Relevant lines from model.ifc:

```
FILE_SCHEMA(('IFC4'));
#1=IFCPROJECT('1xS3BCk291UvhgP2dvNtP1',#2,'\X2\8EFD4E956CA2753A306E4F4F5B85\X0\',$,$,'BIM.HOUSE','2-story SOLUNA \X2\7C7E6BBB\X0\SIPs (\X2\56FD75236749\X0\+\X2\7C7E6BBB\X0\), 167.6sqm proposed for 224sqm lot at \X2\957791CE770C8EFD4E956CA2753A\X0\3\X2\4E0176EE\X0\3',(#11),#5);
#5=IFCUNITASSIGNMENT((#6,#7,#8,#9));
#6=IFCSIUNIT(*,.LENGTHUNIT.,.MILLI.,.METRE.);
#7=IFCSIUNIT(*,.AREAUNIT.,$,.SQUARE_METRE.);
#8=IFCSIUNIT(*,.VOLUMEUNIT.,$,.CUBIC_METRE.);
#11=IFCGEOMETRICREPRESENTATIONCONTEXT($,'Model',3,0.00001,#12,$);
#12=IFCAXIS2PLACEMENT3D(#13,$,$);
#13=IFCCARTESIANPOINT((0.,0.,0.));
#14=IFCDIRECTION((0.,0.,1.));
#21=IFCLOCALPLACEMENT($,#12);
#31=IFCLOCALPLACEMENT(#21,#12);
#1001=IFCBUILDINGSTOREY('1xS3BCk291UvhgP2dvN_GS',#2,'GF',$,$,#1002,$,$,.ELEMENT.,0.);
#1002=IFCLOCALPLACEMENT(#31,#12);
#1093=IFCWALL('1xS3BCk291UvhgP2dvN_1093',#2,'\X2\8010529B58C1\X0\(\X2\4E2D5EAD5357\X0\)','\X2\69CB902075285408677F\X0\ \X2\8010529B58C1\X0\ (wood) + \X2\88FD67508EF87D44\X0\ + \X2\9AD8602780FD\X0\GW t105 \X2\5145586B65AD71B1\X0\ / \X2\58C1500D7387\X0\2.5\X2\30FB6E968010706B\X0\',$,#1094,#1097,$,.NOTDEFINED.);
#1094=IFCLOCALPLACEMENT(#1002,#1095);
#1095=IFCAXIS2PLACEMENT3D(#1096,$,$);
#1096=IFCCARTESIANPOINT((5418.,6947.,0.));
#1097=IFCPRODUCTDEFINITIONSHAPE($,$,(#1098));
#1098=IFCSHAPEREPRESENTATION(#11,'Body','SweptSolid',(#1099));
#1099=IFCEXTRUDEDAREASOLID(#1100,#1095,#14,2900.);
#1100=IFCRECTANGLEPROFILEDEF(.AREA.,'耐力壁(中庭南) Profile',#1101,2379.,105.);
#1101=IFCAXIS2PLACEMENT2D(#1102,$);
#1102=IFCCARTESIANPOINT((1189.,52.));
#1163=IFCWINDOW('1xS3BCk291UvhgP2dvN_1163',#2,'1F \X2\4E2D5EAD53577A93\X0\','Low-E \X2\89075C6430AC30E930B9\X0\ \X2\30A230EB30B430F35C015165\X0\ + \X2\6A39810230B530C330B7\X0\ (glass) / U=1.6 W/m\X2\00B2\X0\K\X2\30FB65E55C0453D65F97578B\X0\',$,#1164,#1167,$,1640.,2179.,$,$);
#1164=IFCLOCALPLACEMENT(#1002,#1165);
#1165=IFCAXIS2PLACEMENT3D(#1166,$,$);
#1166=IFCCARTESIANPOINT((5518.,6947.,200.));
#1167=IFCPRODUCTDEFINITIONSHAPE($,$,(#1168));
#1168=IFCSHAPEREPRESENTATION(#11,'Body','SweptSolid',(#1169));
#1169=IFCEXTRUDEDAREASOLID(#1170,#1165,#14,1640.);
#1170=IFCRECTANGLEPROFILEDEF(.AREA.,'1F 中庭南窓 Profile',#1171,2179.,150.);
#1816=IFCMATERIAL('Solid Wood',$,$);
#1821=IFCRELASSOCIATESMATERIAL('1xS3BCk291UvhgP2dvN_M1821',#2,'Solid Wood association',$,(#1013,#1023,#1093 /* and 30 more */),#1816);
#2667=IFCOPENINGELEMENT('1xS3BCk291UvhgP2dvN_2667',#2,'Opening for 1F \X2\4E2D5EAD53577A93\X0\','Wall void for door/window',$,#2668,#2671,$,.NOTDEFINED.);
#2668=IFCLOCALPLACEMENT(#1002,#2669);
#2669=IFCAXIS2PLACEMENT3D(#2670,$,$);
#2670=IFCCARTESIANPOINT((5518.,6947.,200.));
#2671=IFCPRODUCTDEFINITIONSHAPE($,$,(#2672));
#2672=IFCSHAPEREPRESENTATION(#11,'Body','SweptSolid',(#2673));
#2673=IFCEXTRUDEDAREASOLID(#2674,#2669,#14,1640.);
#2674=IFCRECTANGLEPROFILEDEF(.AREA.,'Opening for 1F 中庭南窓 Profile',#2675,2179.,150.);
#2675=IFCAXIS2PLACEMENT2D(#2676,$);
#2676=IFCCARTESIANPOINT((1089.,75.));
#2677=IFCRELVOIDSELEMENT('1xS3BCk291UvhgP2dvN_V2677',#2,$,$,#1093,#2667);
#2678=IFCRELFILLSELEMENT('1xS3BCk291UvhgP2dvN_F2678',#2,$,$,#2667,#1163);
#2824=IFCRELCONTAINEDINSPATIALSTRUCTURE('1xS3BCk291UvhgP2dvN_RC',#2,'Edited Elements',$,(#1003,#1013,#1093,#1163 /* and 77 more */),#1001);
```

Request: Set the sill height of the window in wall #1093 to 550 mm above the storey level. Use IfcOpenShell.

```python
import numpy as np
import ifcopenshell
import ifcopenshell.api.geometry
import ifcopenshell.geom
import ifcopenshell.util.element
import ifcopenshell.util.placement
import ifcopenshell.util.shape
import ifcopenshell.util.unit

model = ifcopenshell.open("model.ifc")
unit_scale = ifcopenshell.util.unit.calculate_unit_scale(model)

window = model.by_guid("1xS3BCk291UvhgP2dvN_1163")
opening = window.FillsVoids[0].RelatingOpeningElement
storey = ifcopenshell.util.element.get_container(window, ifc_class="IfcBuildingStorey")
level = ifcopenshell.util.placement.get_local_placement(storey.ObjectPlacement)[2, 3]

# The opening's origin need not be at the sill, so measure its lowest point.
shape = ifcopenshell.geom.create_shape(ifcopenshell.geom.settings(), opening)
bottom = ifcopenshell.util.shape.get_shape_bottom_elevation(shape, shape.geometry) / unit_scale
dz = level + 550.0 - bottom

shift = np.array([0.0, 0.0, dz])
# The window is not placed relative to its opening, so move both.
for product in (opening, window):
    matrix = ifcopenshell.util.placement.get_local_placement(product.ObjectPlacement)
    matrix[:3, 3] += shift
    ifcopenshell.api.geometry.edit_object_placement(model, product=product, matrix=matrix, is_si=False)

print(f"moved by {dz * unit_scale:+.3f} m")

model.write("model_updated.ifc")
```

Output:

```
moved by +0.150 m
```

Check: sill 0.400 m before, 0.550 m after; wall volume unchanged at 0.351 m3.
